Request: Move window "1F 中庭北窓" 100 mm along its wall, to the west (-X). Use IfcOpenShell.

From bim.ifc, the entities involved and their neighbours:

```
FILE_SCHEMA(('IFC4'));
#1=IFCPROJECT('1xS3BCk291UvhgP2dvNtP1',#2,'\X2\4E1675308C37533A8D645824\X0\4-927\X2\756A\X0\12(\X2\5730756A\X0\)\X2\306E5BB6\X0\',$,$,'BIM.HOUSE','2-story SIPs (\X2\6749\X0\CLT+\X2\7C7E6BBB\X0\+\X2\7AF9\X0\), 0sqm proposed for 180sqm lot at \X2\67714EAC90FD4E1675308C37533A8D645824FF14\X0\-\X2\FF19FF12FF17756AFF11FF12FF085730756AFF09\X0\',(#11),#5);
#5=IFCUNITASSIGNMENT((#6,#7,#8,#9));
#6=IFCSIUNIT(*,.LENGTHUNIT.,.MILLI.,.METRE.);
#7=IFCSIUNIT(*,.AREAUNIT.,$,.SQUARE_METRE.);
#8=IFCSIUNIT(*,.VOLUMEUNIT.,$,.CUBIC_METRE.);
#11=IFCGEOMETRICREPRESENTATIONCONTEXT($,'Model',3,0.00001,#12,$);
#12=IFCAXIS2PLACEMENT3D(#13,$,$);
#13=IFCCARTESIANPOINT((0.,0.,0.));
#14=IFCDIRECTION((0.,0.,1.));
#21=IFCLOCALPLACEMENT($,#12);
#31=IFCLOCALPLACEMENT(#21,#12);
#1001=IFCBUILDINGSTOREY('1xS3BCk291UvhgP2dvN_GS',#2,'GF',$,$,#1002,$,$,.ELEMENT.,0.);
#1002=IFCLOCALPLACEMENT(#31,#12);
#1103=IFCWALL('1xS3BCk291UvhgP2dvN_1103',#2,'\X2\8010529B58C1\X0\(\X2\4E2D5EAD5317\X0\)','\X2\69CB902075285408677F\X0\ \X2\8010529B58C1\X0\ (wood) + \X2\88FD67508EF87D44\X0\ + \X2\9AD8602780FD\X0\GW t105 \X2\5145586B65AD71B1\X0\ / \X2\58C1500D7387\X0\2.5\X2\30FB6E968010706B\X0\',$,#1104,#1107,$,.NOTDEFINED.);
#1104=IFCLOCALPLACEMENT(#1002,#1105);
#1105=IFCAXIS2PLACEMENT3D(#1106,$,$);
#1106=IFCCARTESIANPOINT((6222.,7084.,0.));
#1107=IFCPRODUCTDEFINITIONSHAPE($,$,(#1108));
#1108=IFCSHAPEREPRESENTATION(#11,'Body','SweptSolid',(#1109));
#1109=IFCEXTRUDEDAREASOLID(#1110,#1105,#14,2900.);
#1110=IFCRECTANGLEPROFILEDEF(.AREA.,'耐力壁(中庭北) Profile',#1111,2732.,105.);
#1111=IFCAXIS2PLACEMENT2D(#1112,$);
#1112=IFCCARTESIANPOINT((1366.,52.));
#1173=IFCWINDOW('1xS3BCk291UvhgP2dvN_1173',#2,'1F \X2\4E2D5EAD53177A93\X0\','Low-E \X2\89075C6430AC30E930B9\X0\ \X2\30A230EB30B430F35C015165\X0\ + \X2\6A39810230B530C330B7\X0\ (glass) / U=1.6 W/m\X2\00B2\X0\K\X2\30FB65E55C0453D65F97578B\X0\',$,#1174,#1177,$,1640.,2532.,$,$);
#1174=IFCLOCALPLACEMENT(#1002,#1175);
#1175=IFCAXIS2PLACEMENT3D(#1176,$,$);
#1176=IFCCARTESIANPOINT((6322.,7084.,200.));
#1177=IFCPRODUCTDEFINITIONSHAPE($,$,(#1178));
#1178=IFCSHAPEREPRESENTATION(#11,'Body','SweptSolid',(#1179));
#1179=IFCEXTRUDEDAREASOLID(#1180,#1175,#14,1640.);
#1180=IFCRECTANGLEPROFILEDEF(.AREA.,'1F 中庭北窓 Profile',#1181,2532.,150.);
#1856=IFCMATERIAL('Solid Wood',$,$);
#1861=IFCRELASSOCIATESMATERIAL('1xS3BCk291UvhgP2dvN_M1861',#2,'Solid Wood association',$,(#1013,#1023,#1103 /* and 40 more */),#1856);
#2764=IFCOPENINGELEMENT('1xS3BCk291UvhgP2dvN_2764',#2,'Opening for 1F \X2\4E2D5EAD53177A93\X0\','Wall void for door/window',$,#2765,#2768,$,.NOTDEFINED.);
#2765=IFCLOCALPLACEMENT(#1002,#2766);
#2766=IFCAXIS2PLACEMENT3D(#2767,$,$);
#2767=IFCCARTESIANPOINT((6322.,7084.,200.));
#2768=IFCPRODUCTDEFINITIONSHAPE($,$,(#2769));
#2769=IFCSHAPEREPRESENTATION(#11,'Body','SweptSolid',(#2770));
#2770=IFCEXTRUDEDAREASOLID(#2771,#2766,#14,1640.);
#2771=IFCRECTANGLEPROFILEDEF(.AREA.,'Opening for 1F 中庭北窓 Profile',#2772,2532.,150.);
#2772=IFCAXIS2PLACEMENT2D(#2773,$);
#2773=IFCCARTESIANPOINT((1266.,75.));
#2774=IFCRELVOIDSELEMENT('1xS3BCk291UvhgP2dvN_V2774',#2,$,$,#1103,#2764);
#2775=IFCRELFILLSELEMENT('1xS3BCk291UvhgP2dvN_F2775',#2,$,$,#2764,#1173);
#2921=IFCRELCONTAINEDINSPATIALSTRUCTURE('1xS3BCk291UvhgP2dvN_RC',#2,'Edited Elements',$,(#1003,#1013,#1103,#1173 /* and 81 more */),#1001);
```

```python
import ifcopenshell
import ifcopenshell.api.geometry
import ifcopenshell.util.placement
import ifcopenshell.util.unit

model = ifcopenshell.open("bim.ifc")
unit_scale = ifcopenshell.util.unit.calculate_unit_scale(model)

window = model.by_guid("1xS3BCk291UvhgP2dvN_1173")
opening = window.FillsVoids[0].RelatingOpeningElement
wall = opening.VoidsElements[0].RelatingBuildingElement

wall_matrix = ifcopenshell.util.placement.get_local_placement(wall.ObjectPlacement)
shift = wall_matrix[:3, 0] * -0.1 / unit_scale
before = ifcopenshell.util.placement.get_local_placement(window.ObjectPlacement)[:3, 3].copy()

# The window is not placed relative to its opening, so move both.
for product in (opening, window):
    matrix = ifcopenshell.util.placement.get_local_placement(product.ObjectPlacement)
    matrix[:3, 3] += shift
    ifcopenshell.api.geometry.edit_object_placement(model, product=product, matrix=matrix, is_si=False)

after = ifcopenshell.util.placement.get_local_placement(window.ObjectPlacement)[:3, 3]
print("window moved by", (after - before).round(3) + 0.0)

model.write("bim_rev.ifc")
```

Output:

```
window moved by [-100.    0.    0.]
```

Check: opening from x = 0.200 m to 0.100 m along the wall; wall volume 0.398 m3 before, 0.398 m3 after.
